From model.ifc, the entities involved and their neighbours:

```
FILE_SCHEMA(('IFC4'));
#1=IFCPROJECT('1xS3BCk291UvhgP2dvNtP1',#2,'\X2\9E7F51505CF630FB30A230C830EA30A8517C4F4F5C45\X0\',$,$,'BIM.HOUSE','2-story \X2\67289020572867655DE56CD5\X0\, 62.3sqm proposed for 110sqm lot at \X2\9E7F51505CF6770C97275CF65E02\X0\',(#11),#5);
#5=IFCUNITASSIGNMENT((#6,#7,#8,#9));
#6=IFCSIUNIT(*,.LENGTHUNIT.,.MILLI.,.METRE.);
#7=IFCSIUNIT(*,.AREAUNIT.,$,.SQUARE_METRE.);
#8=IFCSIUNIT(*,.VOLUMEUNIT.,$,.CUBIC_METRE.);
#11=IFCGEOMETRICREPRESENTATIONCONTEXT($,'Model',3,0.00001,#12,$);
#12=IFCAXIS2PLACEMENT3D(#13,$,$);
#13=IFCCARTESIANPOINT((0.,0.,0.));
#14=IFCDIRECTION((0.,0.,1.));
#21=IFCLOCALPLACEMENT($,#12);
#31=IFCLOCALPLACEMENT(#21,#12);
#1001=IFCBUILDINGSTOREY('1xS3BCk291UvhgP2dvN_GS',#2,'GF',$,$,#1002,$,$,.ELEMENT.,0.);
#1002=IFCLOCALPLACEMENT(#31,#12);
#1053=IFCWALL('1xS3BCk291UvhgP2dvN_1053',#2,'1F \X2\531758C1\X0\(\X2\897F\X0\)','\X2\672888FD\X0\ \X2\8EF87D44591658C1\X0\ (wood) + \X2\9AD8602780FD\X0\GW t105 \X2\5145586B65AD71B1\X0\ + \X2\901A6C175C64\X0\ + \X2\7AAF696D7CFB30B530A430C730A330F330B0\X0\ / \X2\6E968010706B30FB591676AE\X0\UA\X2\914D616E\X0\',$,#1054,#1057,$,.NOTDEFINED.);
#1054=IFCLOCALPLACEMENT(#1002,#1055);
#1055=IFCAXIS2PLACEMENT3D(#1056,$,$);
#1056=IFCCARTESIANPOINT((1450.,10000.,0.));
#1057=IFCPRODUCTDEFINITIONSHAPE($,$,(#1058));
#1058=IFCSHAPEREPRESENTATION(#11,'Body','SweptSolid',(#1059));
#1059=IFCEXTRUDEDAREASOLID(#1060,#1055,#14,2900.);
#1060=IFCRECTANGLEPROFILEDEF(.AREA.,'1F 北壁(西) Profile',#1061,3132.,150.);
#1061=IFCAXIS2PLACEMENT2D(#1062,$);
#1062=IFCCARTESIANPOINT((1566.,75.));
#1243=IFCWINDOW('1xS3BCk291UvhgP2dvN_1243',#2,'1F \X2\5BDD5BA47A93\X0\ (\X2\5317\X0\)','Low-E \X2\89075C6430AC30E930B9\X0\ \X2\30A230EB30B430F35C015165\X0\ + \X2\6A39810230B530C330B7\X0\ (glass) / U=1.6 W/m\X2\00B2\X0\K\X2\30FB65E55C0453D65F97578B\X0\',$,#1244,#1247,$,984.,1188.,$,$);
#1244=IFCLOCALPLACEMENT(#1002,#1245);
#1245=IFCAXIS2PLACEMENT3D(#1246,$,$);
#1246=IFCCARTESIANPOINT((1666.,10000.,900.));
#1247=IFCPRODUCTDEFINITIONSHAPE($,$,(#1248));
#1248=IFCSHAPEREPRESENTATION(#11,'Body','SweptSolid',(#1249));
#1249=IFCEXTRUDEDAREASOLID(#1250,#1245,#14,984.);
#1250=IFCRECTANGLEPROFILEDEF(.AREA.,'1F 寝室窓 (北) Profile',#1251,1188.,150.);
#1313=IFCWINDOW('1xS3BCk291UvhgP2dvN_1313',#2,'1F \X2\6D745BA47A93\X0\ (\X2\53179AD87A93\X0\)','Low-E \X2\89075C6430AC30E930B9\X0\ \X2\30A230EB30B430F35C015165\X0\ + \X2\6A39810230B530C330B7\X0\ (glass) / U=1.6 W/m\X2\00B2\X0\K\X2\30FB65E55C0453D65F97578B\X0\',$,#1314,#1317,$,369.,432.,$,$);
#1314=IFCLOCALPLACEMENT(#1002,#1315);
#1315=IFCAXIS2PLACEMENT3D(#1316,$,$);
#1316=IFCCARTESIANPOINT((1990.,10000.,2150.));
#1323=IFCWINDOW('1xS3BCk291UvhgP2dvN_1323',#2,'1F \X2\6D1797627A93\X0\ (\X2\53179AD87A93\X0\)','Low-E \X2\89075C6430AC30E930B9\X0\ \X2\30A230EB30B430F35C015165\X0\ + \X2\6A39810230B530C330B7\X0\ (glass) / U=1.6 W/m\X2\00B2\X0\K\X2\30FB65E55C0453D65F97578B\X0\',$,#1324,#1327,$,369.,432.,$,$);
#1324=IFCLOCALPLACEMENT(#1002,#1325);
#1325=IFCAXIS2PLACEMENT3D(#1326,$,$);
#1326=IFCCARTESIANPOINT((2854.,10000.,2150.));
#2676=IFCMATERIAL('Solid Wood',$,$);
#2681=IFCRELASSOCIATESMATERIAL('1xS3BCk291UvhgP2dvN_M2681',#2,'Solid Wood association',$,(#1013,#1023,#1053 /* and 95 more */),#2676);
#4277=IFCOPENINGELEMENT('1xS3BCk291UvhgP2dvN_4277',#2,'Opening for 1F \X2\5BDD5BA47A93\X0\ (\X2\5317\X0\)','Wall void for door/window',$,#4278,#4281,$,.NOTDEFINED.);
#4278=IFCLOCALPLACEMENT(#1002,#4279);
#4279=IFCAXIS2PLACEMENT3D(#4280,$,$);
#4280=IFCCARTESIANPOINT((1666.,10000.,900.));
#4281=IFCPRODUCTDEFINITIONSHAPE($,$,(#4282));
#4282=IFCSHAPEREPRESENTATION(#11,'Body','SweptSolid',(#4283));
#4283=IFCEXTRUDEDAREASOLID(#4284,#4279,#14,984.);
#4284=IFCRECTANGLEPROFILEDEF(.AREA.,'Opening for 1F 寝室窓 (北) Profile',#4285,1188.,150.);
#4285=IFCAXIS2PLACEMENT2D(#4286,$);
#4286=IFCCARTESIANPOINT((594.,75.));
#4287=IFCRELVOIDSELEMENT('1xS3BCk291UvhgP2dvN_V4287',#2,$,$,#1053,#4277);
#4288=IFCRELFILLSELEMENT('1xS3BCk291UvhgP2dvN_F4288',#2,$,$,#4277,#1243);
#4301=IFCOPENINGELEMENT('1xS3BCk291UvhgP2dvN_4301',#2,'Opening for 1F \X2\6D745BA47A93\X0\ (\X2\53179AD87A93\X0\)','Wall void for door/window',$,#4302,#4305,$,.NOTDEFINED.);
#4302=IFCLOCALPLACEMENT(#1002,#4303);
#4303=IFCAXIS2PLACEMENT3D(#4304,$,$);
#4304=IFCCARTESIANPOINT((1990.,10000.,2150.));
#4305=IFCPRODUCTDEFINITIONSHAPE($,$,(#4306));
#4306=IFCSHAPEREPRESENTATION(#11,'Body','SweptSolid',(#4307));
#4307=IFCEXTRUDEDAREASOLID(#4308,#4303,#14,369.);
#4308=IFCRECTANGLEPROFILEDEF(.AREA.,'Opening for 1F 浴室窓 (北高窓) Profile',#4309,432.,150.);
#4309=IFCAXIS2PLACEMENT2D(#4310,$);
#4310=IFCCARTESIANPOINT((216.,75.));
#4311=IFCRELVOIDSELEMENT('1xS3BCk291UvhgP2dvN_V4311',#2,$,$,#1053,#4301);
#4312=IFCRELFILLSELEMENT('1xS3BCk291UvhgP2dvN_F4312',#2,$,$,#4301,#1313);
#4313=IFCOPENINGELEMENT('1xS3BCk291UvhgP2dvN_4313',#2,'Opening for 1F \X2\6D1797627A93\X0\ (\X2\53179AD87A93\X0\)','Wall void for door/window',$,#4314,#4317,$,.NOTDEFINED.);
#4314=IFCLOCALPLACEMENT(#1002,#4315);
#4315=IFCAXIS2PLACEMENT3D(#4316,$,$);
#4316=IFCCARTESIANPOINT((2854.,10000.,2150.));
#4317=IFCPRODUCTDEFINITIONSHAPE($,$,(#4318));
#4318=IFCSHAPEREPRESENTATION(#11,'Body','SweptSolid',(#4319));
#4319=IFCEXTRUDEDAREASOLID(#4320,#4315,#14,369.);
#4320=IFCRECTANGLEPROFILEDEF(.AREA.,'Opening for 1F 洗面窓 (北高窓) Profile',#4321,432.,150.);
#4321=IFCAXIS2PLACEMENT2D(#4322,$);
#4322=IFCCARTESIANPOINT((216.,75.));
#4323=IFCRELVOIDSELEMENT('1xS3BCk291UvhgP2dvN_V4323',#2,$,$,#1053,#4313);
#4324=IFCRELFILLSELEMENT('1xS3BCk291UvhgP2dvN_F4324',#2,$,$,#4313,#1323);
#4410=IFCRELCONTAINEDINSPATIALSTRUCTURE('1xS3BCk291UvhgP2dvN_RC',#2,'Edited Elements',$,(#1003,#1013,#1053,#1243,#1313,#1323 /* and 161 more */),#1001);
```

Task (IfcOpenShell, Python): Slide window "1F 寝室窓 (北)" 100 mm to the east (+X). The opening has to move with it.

```python
import ifcopenshell
import ifcopenshell.api.geometry
import ifcopenshell.util.placement
import ifcopenshell.util.unit

model = ifcopenshell.open("model.ifc")
unit_scale = ifcopenshell.util.unit.calculate_unit_scale(model)

window = model.by_guid("1xS3BCk291UvhgP2dvN_1243")
opening = window.FillsVoids[0].RelatingOpeningElement
wall = opening.VoidsElements[0].RelatingBuildingElement

wall_matrix = ifcopenshell.util.placement.get_local_placement(wall.ObjectPlacement)
shift = wall_matrix[:3, 0] * 0.1 / unit_scale
before = ifcopenshell.util.placement.get_local_placement(window.ObjectPlacement)[:3, 3].copy()

# The window is not placed relative to its opening, so move both.
for product in (opening, window):
    matrix = ifcopenshell.util.placement.get_local_placement(product.ObjectPlacement)
    matrix[:3, 3] += shift
    ifcopenshell.api.geometry.edit_object_placement(model, product=product, matrix=matrix, is_si=False)

after = ifcopenshell.util.placement.get_local_placement(window.ObjectPlacement)[:3, 3]
print("window moved by", (after - before).round(3) + 0.0)

model.write("model-out.ifc")
```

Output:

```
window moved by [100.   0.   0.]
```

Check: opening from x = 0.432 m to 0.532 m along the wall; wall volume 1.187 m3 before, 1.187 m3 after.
